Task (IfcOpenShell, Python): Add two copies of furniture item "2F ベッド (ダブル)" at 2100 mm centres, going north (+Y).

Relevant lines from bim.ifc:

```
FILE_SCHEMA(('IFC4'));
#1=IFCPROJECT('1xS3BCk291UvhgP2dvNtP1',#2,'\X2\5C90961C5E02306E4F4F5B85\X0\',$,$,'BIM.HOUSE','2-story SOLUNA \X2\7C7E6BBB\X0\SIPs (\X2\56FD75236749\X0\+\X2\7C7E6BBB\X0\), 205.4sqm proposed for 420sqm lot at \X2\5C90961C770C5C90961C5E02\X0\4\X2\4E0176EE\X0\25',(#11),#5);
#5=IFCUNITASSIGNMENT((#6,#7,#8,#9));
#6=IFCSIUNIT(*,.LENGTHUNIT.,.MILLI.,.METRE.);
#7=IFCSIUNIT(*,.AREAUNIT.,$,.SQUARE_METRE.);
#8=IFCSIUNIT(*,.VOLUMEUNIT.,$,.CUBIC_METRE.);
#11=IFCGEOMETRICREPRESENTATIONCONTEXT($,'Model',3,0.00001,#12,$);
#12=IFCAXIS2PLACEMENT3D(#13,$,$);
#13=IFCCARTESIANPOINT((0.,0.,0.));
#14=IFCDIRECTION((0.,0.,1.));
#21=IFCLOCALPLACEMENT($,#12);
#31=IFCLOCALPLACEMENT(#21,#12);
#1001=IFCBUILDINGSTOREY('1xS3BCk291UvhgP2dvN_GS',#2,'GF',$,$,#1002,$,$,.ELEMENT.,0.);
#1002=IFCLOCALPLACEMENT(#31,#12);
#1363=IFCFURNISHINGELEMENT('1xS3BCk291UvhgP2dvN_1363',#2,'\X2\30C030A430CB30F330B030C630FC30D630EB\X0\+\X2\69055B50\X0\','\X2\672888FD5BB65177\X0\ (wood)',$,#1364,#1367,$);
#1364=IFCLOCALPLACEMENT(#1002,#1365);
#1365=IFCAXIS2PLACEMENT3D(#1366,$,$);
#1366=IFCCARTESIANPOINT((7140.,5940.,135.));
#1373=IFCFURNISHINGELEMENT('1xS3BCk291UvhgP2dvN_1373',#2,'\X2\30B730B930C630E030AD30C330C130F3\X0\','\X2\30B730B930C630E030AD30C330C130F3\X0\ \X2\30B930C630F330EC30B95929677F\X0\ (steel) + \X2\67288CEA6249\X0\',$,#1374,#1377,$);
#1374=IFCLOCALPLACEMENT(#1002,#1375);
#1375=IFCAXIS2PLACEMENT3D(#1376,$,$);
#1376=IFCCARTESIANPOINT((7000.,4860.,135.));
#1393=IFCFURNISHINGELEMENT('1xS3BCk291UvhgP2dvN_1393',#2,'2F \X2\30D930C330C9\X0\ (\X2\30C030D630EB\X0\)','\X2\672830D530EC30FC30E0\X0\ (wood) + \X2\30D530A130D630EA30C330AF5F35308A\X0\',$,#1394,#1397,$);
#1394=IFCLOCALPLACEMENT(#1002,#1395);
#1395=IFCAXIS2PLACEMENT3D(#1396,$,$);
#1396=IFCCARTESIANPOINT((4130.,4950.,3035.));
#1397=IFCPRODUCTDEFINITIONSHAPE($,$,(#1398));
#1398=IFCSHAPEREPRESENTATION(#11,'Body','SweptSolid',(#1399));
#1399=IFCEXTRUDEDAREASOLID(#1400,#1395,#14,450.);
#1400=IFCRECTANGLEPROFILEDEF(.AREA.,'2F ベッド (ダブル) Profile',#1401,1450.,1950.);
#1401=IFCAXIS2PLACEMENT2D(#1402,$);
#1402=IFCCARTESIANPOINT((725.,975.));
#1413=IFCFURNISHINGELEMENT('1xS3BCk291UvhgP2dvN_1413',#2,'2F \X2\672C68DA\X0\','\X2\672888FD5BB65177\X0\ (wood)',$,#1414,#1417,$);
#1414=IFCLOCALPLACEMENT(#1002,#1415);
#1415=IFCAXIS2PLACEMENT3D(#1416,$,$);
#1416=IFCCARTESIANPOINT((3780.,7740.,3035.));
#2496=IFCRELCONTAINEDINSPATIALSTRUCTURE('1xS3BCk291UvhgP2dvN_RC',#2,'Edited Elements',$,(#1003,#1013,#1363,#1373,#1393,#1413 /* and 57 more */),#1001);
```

```python
import numpy as np
import ifcopenshell
import ifcopenshell.api.geometry
import ifcopenshell.api.root
import ifcopenshell.util.element
import ifcopenshell.util.placement
import ifcopenshell.util.unit

model = ifcopenshell.open("bim.ifc")
unit_scale = ifcopenshell.util.unit.calculate_unit_scale(model)


def reuse_history(source, copy):
    """copy_class also copies each property set's owner history, people and application; keep the originals."""
    for rel in copy.IsDefinedBy:
        if rel.is_a("IfcRelDefinesByProperties") and (history := rel.RelatingPropertyDefinition.OwnerHistory):
            rel.RelatingPropertyDefinition.OwnerHistory = source.OwnerHistory
            ifcopenshell.util.element.remove_deep2(model, history)


source = model.by_guid("1xS3BCk291UvhgP2dvN_1393")
base = ifcopenshell.util.placement.get_local_placement(source.ObjectPlacement)
step = np.array([0.0, 1.0, 0.0]) * 2.1 / unit_scale

for i in range(1, 3):
    copy = ifcopenshell.api.root.copy_class(model, product=source)
    copy.Representation = ifcopenshell.util.element.copy_deep(
        model, source.Representation, exclude=["IfcGeometricRepresentationContext", "IfcRepresentationMap"]
    )
    reuse_history(source, copy)
    matrix = base.copy()
    matrix[:3, 3] += i * step
    print("added at", matrix[:3, 3].round(3) + 0.0)
    ifcopenshell.api.geometry.edit_object_placement(model, product=copy, matrix=matrix, is_si=False)

model.write("bim_v2.ifc")
```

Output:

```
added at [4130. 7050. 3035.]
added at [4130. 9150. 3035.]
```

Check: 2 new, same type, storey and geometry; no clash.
